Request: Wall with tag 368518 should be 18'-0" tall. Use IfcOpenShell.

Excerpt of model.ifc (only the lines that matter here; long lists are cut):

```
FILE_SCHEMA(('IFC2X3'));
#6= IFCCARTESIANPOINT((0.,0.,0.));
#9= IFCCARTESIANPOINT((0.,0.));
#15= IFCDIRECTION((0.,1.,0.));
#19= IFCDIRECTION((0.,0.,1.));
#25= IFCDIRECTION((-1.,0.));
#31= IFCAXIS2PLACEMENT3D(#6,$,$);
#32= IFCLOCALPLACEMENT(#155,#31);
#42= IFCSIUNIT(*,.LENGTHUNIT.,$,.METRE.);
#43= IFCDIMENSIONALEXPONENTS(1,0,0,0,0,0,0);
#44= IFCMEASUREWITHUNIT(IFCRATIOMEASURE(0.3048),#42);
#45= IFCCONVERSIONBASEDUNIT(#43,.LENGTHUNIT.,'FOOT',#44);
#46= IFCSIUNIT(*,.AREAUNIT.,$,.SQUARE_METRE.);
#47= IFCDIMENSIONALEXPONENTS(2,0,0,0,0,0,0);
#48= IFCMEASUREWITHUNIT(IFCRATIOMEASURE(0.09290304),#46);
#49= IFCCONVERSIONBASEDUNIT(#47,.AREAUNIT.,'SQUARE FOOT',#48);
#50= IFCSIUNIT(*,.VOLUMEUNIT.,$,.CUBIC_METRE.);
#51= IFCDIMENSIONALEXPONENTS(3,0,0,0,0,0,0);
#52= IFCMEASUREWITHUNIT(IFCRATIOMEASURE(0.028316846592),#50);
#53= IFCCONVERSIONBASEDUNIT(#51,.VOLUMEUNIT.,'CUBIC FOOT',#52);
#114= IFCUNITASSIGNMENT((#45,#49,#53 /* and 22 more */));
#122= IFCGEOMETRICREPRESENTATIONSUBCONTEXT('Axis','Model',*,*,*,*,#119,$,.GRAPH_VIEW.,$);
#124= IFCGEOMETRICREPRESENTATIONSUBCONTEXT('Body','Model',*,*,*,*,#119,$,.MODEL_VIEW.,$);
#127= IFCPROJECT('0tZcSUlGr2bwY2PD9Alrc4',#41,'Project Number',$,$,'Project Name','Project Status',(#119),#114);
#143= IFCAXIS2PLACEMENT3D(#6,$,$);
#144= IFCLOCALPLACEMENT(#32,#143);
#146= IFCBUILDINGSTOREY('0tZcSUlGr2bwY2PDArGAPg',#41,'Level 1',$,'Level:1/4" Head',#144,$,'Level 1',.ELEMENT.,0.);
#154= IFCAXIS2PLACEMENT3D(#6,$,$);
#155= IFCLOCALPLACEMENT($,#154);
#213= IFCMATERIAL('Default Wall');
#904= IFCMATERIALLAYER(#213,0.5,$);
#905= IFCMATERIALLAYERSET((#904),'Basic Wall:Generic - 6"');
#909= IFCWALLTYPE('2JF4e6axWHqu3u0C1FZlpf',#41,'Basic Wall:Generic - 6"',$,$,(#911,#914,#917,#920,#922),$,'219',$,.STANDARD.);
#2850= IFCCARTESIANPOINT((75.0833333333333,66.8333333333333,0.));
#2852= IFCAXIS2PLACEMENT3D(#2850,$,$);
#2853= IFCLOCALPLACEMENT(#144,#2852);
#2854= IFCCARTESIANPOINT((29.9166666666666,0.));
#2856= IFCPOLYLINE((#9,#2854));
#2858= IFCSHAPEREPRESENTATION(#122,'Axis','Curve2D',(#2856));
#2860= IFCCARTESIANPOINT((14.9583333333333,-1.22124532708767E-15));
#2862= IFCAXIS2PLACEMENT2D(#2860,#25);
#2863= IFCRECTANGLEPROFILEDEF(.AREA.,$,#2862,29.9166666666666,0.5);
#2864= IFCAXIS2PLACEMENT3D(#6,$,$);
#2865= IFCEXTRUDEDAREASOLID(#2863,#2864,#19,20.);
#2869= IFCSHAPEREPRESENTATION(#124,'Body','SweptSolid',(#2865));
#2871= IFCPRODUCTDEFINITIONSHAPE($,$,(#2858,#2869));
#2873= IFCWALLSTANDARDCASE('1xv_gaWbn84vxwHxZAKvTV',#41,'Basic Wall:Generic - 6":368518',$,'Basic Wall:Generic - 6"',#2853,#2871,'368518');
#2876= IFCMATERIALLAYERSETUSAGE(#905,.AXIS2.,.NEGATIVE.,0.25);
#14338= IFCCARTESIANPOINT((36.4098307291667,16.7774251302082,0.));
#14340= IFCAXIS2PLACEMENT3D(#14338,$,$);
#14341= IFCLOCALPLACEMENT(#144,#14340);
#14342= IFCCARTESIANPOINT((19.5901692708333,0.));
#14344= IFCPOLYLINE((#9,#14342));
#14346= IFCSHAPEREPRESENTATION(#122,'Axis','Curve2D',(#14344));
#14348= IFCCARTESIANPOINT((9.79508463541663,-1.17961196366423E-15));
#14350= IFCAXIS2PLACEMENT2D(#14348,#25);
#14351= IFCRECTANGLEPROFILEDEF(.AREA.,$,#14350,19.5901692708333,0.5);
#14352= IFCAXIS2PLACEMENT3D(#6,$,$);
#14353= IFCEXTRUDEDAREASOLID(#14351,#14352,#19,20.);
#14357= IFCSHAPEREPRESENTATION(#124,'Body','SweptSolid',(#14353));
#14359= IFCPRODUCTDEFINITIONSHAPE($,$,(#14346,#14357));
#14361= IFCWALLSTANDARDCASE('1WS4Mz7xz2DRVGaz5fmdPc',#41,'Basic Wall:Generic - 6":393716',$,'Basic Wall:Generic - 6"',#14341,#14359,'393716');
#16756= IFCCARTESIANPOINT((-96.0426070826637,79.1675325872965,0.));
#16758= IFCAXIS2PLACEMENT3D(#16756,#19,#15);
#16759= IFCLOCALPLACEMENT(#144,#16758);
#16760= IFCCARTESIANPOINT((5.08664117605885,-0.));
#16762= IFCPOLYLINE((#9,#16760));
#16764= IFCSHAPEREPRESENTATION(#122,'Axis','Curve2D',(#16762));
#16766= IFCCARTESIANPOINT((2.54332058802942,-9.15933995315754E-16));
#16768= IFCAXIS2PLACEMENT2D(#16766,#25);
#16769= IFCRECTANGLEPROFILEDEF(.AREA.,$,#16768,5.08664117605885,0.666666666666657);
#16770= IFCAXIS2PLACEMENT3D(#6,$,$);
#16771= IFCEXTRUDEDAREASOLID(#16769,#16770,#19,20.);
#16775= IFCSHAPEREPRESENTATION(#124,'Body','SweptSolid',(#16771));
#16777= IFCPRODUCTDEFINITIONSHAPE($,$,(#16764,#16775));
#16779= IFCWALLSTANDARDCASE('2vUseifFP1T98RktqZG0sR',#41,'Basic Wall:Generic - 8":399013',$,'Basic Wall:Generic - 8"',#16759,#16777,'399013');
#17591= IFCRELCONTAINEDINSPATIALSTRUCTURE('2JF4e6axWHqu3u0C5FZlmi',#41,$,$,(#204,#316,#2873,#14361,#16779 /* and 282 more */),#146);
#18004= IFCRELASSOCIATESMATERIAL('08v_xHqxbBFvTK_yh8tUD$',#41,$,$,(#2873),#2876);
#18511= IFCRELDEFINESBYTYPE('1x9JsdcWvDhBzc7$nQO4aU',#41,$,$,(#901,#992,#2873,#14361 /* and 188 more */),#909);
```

```python
import ifcopenshell
import ifcopenshell.geom
import ifcopenshell.util.representation
import ifcopenshell.util.shape
import ifcopenshell.util.unit

model = ifcopenshell.open("model.ifc")
unit_scale = ifcopenshell.util.unit.calculate_unit_scale(model)
settings = ifcopenshell.geom.settings()


def volume(element):
    """Net volume in cubic metres, openings subtracted."""
    shape = ifcopenshell.geom.create_shape(settings, element)
    return ifcopenshell.util.shape.get_volume(shape.geometry)


wall = model.by_guid("1xv_gaWbn84vxwHxZAKvTV")
before = volume(wall)

body = ifcopenshell.util.representation.get_representation(wall, "Model", "Body")
solid = body.Items[0]
old_height = solid.Depth
solid.Depth = 216 * 0.0254 / unit_scale
after = volume(wall)

print(f"height {old_height:g} -> {solid.Depth:g}, volume {before:.3f} -> {after:.3f} m3")

model.write("model-out.ifc")
```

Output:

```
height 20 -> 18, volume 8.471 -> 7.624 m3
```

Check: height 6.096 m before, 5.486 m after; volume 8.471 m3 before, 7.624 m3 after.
